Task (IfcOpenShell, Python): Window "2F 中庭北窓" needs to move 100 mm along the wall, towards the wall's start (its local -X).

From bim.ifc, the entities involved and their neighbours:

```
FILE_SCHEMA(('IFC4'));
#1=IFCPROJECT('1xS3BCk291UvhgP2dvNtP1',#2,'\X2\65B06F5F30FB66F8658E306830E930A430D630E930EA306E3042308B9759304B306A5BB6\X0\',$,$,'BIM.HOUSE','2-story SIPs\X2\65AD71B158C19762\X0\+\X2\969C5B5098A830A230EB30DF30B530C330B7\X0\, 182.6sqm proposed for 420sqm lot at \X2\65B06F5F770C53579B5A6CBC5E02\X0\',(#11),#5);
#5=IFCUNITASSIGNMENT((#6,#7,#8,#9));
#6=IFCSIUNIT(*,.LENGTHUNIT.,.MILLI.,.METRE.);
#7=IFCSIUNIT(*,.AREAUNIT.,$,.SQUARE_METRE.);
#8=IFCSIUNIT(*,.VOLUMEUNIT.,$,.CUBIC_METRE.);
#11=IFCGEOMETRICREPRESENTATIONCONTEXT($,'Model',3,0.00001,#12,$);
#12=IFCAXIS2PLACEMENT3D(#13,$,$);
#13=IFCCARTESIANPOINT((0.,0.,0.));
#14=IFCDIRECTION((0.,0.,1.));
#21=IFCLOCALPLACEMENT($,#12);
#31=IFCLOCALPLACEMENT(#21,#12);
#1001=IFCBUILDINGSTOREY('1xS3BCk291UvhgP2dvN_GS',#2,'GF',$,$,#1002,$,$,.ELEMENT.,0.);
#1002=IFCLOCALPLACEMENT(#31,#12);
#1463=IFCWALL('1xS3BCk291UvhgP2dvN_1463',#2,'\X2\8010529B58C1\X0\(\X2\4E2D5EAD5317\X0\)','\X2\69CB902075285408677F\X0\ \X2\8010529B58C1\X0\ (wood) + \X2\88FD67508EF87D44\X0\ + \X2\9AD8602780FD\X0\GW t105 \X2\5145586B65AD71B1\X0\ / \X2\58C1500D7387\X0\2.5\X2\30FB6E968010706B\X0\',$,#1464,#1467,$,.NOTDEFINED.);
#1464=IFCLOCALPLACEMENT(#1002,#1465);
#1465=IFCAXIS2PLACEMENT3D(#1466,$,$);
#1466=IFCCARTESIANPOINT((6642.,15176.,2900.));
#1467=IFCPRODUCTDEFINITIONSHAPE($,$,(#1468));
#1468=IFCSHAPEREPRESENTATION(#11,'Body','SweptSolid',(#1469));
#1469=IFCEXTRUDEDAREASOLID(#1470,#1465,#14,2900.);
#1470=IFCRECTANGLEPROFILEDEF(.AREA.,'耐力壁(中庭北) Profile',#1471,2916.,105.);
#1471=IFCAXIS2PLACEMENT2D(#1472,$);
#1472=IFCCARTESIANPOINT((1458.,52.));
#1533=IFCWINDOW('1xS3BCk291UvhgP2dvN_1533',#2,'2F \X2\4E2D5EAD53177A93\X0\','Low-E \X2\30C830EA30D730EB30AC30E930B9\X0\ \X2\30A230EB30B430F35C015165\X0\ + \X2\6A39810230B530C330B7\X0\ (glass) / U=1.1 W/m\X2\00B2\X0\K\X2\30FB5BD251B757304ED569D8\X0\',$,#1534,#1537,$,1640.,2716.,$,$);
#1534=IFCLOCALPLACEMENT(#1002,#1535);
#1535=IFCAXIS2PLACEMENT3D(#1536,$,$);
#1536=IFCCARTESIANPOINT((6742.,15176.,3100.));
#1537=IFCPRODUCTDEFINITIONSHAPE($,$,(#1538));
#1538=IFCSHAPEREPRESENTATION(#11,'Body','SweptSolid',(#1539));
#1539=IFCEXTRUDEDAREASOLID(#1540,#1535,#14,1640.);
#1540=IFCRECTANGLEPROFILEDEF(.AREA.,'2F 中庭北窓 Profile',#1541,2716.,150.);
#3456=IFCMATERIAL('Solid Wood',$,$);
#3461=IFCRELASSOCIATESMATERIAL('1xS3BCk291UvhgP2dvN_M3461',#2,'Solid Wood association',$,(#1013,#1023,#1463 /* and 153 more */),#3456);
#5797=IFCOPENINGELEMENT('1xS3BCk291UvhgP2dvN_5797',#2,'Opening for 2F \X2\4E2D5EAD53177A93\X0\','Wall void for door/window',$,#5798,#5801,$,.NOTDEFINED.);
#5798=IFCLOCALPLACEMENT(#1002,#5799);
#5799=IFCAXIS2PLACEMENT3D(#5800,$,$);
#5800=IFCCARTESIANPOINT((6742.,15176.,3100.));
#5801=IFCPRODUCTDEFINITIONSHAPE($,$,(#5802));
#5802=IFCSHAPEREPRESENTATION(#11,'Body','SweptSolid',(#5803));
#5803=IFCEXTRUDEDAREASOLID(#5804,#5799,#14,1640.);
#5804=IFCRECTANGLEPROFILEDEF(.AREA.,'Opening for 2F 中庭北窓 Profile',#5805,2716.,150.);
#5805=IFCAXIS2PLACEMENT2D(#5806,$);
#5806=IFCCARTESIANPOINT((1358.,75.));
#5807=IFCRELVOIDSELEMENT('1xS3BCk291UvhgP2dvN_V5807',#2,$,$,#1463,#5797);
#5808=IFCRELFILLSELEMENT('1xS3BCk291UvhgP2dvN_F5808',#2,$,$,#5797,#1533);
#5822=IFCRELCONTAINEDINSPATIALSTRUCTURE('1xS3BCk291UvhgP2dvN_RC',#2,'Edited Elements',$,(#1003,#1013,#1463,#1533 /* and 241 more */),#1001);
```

```python
import ifcopenshell
import ifcopenshell.api.geometry
import ifcopenshell.util.placement
import ifcopenshell.util.unit

model = ifcopenshell.open("bim.ifc")
unit_scale = ifcopenshell.util.unit.calculate_unit_scale(model)

window = model.by_id(1533)
opening = window.FillsVoids[0].RelatingOpeningElement
wall = opening.VoidsElements[0].RelatingBuildingElement

wall_matrix = ifcopenshell.util.placement.get_local_placement(wall.ObjectPlacement)
shift = wall_matrix[:3, 0] * -0.1 / unit_scale
before = ifcopenshell.util.placement.get_local_placement(window.ObjectPlacement)[:3, 3].copy()

# The window is not placed relative to its opening, so move both.
for product in (opening, window):
    matrix = ifcopenshell.util.placement.get_local_placement(product.ObjectPlacement)
    matrix[:3, 3] += shift
    ifcopenshell.api.geometry.edit_object_placement(model, product=product, matrix=matrix, is_si=False)

after = ifcopenshell.util.placement.get_local_placement(window.ObjectPlacement)[:3, 3]
print("window moved by", (after - before).round(3) + 0.0)

model.write("bim_updated.ifc")
```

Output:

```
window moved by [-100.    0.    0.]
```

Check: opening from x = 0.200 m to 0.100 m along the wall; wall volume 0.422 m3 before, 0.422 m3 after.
